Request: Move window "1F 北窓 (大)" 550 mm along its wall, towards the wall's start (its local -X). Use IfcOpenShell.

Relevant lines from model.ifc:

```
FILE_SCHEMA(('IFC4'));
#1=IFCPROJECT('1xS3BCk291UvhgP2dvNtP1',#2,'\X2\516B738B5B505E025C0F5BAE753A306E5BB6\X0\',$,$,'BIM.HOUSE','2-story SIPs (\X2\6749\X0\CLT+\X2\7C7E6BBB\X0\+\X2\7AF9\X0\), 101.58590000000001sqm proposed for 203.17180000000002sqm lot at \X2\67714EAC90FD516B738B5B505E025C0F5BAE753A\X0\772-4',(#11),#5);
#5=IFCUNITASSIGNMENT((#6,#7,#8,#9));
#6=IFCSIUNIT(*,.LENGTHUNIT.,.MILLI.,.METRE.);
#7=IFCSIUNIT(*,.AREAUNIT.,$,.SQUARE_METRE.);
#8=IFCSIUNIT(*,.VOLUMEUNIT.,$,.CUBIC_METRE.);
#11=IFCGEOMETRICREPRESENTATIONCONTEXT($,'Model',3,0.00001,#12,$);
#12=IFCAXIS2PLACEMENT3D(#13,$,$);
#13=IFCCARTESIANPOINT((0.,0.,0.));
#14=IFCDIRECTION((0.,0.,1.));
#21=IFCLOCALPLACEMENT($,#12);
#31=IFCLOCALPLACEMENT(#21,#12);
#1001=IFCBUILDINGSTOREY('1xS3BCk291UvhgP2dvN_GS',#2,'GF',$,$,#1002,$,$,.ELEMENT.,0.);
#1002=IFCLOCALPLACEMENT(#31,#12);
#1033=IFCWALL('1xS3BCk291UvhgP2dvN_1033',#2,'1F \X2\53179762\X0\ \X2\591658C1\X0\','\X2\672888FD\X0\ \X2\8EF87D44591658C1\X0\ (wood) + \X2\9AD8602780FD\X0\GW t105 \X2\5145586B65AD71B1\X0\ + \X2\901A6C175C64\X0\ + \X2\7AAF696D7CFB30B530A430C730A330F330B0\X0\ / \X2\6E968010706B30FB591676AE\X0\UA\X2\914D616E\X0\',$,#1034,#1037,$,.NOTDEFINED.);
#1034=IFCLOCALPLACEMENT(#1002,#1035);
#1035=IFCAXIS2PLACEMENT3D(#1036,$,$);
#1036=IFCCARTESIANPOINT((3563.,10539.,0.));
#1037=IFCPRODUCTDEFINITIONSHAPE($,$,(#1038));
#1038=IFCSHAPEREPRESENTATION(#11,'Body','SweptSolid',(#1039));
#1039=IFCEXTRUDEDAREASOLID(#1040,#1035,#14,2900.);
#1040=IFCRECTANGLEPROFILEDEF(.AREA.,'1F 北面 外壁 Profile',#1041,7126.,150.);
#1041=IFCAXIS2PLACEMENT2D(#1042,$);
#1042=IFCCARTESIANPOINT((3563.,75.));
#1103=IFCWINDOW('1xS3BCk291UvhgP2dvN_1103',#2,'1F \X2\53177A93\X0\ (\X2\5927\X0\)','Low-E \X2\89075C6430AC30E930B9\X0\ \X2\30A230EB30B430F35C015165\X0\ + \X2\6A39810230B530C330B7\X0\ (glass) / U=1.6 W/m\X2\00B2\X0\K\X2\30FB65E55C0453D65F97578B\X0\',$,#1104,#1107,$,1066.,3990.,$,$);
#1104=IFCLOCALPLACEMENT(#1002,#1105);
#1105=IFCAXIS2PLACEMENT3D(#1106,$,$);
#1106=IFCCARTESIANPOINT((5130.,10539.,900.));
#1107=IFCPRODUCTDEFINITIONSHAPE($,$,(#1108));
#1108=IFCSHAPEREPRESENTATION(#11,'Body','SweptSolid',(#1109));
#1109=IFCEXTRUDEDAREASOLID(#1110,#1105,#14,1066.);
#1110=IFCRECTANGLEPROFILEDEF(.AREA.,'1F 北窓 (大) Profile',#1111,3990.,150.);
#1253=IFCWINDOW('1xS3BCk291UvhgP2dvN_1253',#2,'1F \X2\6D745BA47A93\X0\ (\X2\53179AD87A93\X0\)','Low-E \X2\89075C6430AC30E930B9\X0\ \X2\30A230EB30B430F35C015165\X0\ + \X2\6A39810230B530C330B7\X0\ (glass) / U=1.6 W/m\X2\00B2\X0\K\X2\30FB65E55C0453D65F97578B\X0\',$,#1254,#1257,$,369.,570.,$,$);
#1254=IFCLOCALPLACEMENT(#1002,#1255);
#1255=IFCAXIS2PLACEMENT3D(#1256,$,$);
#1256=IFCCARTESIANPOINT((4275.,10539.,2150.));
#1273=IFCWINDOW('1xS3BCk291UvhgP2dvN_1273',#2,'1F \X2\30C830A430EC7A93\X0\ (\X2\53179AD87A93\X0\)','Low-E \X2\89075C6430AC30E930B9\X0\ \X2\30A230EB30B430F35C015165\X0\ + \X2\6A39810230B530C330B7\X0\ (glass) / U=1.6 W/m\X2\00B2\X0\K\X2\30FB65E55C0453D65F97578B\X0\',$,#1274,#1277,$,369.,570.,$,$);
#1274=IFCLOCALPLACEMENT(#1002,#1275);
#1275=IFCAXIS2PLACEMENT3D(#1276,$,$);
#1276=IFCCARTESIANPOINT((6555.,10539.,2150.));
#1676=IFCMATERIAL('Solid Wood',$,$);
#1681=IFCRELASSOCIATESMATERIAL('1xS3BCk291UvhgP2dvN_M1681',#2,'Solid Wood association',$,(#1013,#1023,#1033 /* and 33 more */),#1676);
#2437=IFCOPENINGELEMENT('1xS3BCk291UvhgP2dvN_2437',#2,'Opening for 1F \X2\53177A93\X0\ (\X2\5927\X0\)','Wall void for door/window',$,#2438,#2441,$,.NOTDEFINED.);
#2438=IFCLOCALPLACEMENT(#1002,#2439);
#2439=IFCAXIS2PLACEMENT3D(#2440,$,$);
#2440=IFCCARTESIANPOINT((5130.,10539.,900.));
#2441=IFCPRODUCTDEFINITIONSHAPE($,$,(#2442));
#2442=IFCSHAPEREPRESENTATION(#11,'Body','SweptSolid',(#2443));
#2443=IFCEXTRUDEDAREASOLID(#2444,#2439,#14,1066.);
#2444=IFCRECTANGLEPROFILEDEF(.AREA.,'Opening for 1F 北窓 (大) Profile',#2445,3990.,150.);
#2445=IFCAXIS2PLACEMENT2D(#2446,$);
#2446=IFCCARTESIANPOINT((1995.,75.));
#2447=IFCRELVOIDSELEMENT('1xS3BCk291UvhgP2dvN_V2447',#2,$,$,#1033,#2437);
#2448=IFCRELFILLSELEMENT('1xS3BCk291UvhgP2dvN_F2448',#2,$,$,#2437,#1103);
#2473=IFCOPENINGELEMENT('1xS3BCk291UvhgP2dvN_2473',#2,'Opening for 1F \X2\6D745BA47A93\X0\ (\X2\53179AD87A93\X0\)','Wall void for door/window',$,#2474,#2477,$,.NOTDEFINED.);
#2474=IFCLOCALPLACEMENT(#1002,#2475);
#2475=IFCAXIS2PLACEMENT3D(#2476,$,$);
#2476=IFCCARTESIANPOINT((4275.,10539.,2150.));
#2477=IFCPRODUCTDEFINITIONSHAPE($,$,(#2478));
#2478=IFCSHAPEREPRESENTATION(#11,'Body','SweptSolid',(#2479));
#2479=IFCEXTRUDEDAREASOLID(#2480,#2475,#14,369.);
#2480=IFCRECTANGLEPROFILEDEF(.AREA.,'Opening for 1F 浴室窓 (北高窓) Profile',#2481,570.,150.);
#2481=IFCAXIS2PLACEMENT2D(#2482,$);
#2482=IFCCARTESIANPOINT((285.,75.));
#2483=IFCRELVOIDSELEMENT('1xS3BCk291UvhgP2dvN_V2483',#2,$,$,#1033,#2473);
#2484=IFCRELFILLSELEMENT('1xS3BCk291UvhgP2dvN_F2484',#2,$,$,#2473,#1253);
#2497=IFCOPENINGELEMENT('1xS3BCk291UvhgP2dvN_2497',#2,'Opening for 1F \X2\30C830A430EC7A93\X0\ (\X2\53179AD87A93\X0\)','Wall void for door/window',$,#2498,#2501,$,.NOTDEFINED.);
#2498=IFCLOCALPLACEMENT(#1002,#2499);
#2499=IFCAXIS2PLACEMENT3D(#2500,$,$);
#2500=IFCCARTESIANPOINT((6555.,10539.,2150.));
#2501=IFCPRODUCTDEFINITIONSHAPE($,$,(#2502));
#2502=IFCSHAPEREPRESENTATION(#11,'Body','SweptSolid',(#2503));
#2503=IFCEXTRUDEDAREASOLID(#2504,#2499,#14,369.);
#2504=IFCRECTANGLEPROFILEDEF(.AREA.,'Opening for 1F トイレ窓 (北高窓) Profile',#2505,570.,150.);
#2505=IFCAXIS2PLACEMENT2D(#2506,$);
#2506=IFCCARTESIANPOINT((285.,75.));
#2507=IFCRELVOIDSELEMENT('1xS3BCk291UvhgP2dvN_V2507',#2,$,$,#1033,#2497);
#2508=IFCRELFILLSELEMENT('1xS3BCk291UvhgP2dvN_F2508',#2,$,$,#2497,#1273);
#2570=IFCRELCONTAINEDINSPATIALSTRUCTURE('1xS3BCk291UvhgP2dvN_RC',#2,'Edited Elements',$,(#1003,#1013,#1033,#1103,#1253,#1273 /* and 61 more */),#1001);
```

```python
import ifcopenshell
import ifcopenshell.api.geometry
import ifcopenshell.util.placement
import ifcopenshell.util.unit

model = ifcopenshell.open("model.ifc")
unit_scale = ifcopenshell.util.unit.calculate_unit_scale(model)

window = model.by_guid("1xS3BCk291UvhgP2dvN_1103")
opening = window.FillsVoids[0].RelatingOpeningElement
wall = opening.VoidsElements[0].RelatingBuildingElement

wall_matrix = ifcopenshell.util.placement.get_local_placement(wall.ObjectPlacement)
shift = wall_matrix[:3, 0] * -0.55 / unit_scale
before = ifcopenshell.util.placement.get_local_placement(window.ObjectPlacement)[:3, 3].copy()

# The window is not placed relative to its opening, so move both.
for product in (opening, window):
    matrix = ifcopenshell.util.placement.get_local_placement(product.ObjectPlacement)
    matrix[:3, 3] += shift
    ifcopenshell.api.geometry.edit_object_placement(model, product=product, matrix=matrix, is_si=False)

after = ifcopenshell.util.placement.get_local_placement(window.ObjectPlacement)[:3, 3]
print("window moved by", (after - before).round(3) + 0.0)

model.write("model_updated.ifc")
```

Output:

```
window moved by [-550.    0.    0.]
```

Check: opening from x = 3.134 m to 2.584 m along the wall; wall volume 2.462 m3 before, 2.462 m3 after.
